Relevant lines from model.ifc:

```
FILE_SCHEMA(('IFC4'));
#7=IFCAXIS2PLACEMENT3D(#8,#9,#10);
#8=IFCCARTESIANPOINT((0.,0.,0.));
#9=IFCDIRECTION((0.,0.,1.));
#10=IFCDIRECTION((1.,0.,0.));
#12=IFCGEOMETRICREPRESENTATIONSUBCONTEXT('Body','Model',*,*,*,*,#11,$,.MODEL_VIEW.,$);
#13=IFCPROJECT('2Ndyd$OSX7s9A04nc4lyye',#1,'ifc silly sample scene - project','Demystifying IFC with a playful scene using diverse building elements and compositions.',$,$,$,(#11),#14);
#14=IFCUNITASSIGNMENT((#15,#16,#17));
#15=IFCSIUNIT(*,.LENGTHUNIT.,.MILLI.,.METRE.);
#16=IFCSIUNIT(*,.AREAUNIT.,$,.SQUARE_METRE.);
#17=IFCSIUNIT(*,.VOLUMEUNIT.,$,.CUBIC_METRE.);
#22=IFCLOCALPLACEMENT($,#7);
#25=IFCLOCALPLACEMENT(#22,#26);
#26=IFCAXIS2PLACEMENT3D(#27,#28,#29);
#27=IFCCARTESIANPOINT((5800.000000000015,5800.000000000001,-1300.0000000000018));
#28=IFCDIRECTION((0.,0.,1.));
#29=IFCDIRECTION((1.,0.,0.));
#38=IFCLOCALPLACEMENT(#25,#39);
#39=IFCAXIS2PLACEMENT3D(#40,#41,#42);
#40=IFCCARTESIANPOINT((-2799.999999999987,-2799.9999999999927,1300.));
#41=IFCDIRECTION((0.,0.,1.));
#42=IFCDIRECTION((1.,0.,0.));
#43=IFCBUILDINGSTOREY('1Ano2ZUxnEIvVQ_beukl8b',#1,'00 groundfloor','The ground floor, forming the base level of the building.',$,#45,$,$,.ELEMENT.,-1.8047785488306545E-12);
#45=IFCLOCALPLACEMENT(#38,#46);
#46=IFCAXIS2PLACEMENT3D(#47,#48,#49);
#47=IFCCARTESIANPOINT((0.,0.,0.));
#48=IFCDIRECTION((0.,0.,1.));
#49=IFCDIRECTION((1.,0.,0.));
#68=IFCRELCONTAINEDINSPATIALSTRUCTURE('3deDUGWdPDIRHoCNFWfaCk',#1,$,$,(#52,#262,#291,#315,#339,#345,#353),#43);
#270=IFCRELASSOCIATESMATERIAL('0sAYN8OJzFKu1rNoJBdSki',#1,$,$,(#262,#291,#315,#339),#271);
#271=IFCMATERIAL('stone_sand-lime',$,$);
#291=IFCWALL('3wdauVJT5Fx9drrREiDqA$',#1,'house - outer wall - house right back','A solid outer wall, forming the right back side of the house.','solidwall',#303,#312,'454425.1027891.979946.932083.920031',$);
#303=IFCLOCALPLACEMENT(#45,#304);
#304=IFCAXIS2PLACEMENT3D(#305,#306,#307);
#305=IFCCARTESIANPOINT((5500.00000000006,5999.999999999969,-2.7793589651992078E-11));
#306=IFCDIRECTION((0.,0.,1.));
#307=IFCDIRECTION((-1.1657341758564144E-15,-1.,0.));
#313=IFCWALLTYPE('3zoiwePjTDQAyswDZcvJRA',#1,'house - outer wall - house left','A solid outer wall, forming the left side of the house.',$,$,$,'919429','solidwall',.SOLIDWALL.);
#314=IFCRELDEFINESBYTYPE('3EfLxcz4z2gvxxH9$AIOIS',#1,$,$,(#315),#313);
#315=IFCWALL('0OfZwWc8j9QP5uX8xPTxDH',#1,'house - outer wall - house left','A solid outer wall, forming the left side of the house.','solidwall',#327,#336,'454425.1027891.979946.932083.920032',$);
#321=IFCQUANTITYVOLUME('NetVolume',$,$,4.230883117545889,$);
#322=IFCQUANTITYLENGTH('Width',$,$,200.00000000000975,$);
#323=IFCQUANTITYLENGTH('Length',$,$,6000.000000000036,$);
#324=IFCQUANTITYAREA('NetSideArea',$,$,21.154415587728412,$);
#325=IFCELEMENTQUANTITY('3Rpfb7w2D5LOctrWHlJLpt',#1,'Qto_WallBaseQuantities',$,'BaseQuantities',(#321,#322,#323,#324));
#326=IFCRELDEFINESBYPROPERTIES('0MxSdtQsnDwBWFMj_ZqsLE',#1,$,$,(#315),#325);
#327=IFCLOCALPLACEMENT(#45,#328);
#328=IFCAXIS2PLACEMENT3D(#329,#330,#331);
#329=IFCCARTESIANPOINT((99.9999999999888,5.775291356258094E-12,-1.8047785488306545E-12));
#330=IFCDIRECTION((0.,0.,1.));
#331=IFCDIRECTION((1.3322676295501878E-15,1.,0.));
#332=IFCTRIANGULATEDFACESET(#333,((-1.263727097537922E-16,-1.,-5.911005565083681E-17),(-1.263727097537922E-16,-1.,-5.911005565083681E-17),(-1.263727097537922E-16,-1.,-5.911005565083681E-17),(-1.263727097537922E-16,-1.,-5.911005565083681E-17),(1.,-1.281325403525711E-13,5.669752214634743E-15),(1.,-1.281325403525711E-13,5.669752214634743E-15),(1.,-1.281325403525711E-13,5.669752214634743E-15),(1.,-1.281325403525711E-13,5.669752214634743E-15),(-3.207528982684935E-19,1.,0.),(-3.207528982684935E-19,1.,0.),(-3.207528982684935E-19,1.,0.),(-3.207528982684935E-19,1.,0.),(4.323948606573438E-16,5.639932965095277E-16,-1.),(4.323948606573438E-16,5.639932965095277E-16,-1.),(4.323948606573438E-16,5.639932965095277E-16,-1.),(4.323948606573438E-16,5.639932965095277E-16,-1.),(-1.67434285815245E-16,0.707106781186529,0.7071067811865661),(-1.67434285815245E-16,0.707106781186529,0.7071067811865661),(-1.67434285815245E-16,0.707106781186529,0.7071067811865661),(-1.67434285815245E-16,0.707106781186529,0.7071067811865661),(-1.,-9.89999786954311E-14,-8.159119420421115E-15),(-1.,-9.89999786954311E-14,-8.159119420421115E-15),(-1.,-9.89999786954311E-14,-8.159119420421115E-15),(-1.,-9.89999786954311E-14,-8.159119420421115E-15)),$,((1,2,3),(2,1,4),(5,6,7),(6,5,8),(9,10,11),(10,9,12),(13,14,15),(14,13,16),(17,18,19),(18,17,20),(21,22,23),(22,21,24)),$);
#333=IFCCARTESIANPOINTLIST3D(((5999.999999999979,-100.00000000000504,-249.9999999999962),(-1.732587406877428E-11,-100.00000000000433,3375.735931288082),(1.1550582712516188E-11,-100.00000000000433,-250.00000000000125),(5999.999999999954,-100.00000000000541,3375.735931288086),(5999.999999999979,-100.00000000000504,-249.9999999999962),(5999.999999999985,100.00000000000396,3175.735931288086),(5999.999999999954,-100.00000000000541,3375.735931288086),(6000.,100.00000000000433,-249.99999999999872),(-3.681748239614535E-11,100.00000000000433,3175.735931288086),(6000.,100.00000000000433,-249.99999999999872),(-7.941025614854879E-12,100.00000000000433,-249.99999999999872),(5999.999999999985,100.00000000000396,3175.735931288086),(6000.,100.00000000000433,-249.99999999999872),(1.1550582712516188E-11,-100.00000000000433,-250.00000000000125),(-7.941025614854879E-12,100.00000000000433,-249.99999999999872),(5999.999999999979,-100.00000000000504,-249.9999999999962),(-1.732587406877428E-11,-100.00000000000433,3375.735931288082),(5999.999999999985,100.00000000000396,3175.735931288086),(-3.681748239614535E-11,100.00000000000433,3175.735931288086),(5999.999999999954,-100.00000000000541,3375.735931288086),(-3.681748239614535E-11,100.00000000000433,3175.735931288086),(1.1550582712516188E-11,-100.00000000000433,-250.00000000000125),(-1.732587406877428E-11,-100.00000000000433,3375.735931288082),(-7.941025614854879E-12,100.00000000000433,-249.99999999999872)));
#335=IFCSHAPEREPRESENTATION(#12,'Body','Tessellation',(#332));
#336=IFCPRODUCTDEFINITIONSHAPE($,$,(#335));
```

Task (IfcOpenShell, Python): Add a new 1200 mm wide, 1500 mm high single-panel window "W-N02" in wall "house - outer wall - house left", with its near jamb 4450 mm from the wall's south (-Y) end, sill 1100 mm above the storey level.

```python
import numpy as np
import ifcopenshell
import ifcopenshell.api.feature
import ifcopenshell.api.geometry
import ifcopenshell.api.pset
import ifcopenshell.api.root
import ifcopenshell.api.spatial
import ifcopenshell.geom
import ifcopenshell.util.element
import ifcopenshell.util.placement
import ifcopenshell.util.representation
import ifcopenshell.util.shape
import ifcopenshell.util.unit

model = ifcopenshell.open("model.ifc")
unit_scale = ifcopenshell.util.unit.calculate_unit_scale(model)
area_scale = ifcopenshell.util.unit.calculate_unit_scale(model, "AREAUNIT")
volume_scale = ifcopenshell.util.unit.calculate_unit_scale(model, "VOLUMEUNIT")
settings = ifcopenshell.geom.settings()


def volume(element):
    """Net volume in cubic metres, openings subtracted."""
    shape = ifcopenshell.geom.create_shape(settings, element)
    return ifcopenshell.util.shape.get_volume(shape.geometry)


wall = model.by_guid("0OfZwWc8j9QP5uX8xPTxDH")
storey = ifcopenshell.util.element.get_container(wall, ifc_class="IfcBuildingStorey")
context = ifcopenshell.util.representation.get_context(model, "Model", "Body", "MODEL_VIEW")
before = volume(wall)

width, height, from_end, sill = 1.2, 1.5, 4.45, 1.1  # metres

# The wall runs along its own X axis, and the end named is its -X end.
wall_shape = ifcopenshell.geom.create_shape(settings, wall)
x, y, z = ifcopenshell.util.shape.get_vertices(wall_shape.geometry).T
start = x.min() + from_end
face, thickness = float(y.min()), float(y.max() - y.min())
wall_matrix = ifcopenshell.util.placement.get_local_placement(wall.ObjectPlacement)
level = ifcopenshell.util.placement.get_local_placement(storey.ObjectPlacement)[2, 3]


def in_wall(x, y):
    """Placement at x, y metres in the wall's axes, at sill height."""
    matrix = wall_matrix.copy()
    matrix[:, 3] = wall_matrix @ np.array([x / unit_scale, y / unit_scale, 0.0, 1.0])
    matrix[2, 3] = level + sill / unit_scale
    return matrix


# Opening: a box that overshoots both wall faces by 50 mm.
opening = ifcopenshell.api.root.create_entity(model, ifc_class="IfcOpeningElement", predefined_type="OPENING")
box = ifcopenshell.api.geometry.add_wall_representation(
    model, context=context, length=width, height=height, thickness=thickness + 0.1
)
ifcopenshell.api.geometry.assign_representation(model, product=opening, representation=box)
ifcopenshell.api.geometry.edit_object_placement(model, product=opening, matrix=in_wall(start, face - 0.05), is_si=False)
ifcopenshell.api.feature.add_feature(model, feature=opening, element=wall)

window = ifcopenshell.api.root.create_entity(model, ifc_class="IfcWindow", name="W-N02", predefined_type="WINDOW")
window.OverallWidth, window.OverallHeight = width / unit_scale, height / unit_scale
window.PartitioningType = "SINGLE_PANEL"
body = ifcopenshell.api.geometry.add_window_representation(
    model,
    context=context,
    overall_width=window.OverallWidth,
    overall_height=window.OverallHeight,
    partition_type="SINGLE_PANEL",
)
ifcopenshell.api.geometry.assign_representation(model, product=window, representation=body)
ifcopenshell.api.spatial.assign_container(model, products=[window], relating_structure=storey)
ifcopenshell.api.feature.add_filling(model, opening=opening, element=window)

# Centre the window in the wall's thickness.
ifcopenshell.api.geometry.edit_object_placement(model, product=window, matrix=in_wall(start, face), is_si=False)
window_shape = ifcopenshell.geom.create_shape(settings, window)
depth = ifcopenshell.util.shape.get_vertices(window_shape.geometry)[:, 1]
offset = face + thickness / 2 - (depth.min() + depth.max()) / 2
ifcopenshell.api.geometry.edit_object_placement(model, product=window, matrix=in_wall(start, offset), is_si=False)

after = volume(wall)

# Update the wall's stored quantities.
qto = model.by_id(ifcopenshell.util.element.get_pset(wall, "Qto_WallBaseQuantities", should_inherit=False)["id"])
ifcopenshell.api.pset.edit_qto(model, qto=qto, properties={
    "NetVolume": after / volume_scale,
    "NetSideArea": after / thickness / area_scale,
})

print(f"wall volume {before:.3f} -> {after:.3f} m3")

model.write("model-out.ifc")
```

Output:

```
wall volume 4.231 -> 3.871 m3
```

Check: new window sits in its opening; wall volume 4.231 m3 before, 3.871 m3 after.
